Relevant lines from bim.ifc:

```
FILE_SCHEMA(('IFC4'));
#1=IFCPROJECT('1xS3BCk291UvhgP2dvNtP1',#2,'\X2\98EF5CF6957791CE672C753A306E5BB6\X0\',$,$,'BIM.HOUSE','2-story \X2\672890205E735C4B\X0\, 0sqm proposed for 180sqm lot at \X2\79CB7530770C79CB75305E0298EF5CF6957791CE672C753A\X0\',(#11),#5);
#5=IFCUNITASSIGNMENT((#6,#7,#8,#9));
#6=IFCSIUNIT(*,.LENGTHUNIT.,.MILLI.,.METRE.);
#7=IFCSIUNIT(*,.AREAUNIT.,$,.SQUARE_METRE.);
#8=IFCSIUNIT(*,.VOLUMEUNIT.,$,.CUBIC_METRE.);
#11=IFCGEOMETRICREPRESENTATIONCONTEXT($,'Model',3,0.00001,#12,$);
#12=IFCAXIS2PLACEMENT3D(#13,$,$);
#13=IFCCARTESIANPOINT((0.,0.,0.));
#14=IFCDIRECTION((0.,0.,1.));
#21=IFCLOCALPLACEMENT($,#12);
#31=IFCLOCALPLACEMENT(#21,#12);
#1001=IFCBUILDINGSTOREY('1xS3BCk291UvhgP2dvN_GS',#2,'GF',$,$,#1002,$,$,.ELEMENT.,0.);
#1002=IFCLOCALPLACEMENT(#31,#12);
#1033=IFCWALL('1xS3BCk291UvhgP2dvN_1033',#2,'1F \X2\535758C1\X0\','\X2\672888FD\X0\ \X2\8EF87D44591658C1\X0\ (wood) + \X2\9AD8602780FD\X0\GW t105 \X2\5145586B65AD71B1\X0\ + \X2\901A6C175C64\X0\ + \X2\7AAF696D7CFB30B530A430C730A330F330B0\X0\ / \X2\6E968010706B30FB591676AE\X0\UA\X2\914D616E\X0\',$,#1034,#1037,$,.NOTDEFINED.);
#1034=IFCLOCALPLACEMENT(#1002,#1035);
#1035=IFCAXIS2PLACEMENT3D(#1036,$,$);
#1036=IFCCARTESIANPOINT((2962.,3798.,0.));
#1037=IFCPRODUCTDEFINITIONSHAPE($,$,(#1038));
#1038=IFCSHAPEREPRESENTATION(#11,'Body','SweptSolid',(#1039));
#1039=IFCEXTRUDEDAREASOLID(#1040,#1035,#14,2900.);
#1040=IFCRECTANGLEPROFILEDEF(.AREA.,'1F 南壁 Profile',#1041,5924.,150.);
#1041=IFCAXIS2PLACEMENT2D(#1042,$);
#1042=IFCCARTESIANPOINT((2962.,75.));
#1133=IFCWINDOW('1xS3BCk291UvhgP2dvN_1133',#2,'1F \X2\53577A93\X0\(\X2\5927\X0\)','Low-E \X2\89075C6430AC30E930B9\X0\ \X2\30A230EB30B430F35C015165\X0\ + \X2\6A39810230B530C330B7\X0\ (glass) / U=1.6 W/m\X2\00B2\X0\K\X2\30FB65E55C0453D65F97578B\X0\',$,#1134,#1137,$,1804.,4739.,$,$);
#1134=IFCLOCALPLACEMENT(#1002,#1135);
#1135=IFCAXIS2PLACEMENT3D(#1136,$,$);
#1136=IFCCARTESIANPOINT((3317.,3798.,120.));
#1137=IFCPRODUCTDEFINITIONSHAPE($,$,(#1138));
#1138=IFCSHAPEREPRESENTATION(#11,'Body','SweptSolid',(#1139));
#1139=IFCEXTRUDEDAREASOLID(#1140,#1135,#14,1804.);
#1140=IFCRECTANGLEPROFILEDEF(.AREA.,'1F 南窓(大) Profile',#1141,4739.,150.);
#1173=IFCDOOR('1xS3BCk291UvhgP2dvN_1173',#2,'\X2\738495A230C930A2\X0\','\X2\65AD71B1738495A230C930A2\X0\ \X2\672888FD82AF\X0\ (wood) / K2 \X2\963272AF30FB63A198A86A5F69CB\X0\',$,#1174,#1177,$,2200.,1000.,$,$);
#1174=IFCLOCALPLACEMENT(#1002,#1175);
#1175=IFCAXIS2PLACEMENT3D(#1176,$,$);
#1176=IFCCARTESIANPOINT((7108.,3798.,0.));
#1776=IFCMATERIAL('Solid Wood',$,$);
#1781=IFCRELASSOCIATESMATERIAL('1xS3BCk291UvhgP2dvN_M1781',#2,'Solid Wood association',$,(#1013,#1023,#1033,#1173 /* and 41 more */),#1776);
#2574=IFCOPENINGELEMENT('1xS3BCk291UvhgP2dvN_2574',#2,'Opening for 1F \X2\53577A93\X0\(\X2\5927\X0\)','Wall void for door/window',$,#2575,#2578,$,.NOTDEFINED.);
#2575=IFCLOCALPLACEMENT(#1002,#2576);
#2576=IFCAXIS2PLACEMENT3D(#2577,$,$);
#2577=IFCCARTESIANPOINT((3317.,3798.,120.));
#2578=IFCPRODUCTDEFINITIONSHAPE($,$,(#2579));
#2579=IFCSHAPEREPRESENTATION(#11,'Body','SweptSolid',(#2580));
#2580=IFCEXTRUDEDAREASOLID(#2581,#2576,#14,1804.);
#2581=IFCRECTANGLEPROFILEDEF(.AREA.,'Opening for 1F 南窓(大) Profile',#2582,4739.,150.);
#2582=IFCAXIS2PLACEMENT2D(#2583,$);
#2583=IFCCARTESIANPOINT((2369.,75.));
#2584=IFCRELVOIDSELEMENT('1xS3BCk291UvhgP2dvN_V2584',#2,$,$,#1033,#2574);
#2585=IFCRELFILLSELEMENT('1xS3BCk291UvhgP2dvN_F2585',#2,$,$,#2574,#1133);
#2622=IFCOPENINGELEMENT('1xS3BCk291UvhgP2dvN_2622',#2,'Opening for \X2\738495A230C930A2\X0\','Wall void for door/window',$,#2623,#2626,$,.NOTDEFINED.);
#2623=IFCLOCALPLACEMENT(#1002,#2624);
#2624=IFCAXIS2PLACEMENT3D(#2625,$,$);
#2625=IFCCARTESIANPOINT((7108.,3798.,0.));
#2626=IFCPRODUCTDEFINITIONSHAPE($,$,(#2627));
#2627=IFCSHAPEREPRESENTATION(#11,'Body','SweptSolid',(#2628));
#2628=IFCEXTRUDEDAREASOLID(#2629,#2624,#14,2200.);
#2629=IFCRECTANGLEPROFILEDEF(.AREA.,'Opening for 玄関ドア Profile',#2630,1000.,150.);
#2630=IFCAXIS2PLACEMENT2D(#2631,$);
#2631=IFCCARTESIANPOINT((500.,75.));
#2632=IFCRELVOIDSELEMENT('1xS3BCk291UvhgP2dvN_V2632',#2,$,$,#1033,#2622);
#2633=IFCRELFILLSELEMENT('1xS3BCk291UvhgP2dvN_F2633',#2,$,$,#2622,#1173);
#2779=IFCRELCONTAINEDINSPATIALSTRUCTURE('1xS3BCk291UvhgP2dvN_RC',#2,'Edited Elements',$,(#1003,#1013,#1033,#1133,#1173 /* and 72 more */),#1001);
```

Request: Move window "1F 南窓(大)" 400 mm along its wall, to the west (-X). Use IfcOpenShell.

```python
import ifcopenshell
import ifcopenshell.api.geometry
import ifcopenshell.util.placement
import ifcopenshell.util.unit

model = ifcopenshell.open("bim.ifc")
unit_scale = ifcopenshell.util.unit.calculate_unit_scale(model)

window = model.by_guid("1xS3BCk291UvhgP2dvN_1133")
opening = window.FillsVoids[0].RelatingOpeningElement
wall = opening.VoidsElements[0].RelatingBuildingElement

wall_matrix = ifcopenshell.util.placement.get_local_placement(wall.ObjectPlacement)
shift = wall_matrix[:3, 0] * -0.4 / unit_scale
before = ifcopenshell.util.placement.get_local_placement(window.ObjectPlacement)[:3, 3].copy()

# The window is not placed relative to its opening, so move both.
for product in (opening, window):
    matrix = ifcopenshell.util.placement.get_local_placement(product.ObjectPlacement)
    matrix[:3, 3] += shift
    ifcopenshell.api.geometry.edit_object_placement(model, product=product, matrix=matrix, is_si=False)

after = ifcopenshell.util.placement.get_local_placement(window.ObjectPlacement)[:3, 3]
print("window moved by", (after - before).round(3) + 0.0)

model.write("bim_rev.ifc")
```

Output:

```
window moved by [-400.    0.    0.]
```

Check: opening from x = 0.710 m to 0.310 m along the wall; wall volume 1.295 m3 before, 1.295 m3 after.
